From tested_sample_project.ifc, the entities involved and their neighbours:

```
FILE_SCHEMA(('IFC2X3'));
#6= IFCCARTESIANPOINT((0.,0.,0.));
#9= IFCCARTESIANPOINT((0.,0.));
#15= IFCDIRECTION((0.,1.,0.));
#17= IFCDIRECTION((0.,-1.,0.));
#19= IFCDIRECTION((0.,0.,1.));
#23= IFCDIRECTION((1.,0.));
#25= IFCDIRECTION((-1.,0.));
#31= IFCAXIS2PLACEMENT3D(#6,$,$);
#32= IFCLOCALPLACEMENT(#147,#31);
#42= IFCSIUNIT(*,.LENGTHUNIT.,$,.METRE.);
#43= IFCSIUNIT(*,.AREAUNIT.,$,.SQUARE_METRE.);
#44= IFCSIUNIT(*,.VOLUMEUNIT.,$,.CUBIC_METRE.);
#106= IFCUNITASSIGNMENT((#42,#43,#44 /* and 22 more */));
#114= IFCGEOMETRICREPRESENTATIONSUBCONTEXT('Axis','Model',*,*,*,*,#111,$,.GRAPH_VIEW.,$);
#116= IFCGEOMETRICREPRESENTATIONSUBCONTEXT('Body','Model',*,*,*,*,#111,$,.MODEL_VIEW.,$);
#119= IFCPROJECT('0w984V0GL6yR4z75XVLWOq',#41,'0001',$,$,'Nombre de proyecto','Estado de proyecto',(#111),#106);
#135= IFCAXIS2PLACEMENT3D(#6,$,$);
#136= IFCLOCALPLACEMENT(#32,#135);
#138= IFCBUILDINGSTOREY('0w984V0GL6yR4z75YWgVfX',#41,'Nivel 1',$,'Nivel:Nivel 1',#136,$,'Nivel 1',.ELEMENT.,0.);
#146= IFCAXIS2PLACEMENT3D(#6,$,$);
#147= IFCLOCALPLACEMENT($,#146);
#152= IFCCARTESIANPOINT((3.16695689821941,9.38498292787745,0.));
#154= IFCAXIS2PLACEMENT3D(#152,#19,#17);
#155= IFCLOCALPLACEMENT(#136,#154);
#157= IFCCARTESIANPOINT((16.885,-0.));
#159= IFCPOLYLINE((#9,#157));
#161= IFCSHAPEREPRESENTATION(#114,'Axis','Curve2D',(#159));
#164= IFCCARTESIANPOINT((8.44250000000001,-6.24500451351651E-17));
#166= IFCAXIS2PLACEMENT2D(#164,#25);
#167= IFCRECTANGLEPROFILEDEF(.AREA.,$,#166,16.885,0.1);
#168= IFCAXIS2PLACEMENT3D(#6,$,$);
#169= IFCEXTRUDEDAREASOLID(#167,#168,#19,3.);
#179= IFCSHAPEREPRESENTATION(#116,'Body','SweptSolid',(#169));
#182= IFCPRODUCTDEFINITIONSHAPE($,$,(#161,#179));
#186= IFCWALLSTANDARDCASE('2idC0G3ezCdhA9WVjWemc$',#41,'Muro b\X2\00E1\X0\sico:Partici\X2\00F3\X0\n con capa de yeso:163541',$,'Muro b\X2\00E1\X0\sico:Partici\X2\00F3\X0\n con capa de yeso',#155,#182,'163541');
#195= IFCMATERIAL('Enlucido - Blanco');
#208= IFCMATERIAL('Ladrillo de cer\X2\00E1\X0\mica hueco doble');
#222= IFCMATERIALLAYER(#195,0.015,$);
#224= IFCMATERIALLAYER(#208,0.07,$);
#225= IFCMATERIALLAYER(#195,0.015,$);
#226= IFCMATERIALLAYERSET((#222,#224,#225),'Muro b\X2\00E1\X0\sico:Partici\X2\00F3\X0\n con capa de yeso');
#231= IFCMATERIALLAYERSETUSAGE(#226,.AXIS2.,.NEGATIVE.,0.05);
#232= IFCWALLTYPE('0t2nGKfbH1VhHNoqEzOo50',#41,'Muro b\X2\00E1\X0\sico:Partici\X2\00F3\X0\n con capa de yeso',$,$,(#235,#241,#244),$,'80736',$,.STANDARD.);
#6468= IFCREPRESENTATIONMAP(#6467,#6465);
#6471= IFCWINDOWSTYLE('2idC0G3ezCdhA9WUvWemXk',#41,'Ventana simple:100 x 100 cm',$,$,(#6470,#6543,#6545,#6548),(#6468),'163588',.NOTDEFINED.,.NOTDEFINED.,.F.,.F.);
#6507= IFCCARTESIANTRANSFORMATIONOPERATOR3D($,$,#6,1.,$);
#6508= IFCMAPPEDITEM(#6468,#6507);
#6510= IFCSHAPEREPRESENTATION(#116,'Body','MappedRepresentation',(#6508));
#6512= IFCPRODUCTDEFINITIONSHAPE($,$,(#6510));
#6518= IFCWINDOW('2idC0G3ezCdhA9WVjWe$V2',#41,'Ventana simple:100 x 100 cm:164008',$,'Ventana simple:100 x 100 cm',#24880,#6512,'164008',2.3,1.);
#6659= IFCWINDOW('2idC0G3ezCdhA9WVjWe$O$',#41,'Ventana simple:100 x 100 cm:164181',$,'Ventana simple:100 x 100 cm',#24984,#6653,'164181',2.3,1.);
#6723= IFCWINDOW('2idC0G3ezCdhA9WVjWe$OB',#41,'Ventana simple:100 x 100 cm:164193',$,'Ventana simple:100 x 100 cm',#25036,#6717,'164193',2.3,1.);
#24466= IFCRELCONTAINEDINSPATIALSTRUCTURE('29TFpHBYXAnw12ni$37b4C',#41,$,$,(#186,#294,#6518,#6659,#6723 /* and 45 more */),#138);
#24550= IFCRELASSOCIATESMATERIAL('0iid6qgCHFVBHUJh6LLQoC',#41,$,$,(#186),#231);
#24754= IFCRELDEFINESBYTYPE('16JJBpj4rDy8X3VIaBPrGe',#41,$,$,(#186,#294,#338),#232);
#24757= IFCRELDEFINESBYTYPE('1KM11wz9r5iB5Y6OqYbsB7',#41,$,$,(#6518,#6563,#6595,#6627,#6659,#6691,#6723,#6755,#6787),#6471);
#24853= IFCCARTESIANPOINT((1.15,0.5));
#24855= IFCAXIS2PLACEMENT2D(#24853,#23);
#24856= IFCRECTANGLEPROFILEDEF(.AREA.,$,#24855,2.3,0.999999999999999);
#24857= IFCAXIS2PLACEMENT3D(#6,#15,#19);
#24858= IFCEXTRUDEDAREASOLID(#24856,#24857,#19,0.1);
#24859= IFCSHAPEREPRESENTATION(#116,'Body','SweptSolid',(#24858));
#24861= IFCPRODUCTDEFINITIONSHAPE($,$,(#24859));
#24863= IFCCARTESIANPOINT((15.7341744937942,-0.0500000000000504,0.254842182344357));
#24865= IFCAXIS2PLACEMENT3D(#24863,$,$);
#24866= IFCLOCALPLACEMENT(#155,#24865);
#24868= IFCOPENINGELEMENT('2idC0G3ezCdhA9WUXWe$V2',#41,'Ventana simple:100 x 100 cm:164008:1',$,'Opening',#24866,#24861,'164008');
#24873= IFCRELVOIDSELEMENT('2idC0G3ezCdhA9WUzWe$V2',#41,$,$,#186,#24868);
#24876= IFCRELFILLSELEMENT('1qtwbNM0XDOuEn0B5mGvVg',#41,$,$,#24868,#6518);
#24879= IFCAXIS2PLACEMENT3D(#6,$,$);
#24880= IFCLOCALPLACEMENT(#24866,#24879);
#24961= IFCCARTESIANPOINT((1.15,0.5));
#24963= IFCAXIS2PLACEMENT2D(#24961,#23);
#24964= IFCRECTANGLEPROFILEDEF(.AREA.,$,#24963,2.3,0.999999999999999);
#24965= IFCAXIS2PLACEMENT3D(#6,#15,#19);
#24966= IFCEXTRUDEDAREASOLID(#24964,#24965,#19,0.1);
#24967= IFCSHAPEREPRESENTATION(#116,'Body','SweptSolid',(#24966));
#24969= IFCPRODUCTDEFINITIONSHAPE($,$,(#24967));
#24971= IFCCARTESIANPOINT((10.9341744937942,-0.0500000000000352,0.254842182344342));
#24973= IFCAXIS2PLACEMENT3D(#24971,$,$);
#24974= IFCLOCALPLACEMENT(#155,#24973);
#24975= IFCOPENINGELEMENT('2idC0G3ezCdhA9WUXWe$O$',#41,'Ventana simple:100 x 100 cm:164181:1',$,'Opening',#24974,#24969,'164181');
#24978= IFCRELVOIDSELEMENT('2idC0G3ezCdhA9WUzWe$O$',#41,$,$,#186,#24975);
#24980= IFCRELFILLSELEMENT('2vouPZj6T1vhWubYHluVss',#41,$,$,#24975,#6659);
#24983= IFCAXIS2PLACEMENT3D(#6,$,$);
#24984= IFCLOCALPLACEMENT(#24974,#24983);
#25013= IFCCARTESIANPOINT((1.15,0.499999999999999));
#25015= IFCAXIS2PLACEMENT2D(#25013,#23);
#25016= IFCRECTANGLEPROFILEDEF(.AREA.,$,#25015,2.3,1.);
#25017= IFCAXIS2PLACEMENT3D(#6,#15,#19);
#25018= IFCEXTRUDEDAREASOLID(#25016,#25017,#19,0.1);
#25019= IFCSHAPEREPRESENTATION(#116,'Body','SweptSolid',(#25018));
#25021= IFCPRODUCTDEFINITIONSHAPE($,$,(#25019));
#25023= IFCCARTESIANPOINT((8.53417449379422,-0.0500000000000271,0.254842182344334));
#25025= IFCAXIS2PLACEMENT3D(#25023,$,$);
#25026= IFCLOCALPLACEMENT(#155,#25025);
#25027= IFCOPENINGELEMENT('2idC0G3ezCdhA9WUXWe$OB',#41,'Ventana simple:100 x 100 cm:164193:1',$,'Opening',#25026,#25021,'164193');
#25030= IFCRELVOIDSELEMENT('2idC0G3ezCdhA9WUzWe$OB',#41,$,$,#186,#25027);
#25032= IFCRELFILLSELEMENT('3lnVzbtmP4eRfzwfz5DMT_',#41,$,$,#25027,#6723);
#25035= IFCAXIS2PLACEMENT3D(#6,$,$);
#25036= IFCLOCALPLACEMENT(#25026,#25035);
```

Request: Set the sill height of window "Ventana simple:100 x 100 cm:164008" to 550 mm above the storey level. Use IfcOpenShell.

```python
import numpy as np
import ifcopenshell
import ifcopenshell.api.geometry
import ifcopenshell.geom
import ifcopenshell.util.element
import ifcopenshell.util.placement
import ifcopenshell.util.shape
import ifcopenshell.util.unit

model = ifcopenshell.open("tested_sample_project.ifc")
unit_scale = ifcopenshell.util.unit.calculate_unit_scale(model)

window = model.by_guid("2idC0G3ezCdhA9WVjWe$V2")
opening = window.FillsVoids[0].RelatingOpeningElement
storey = ifcopenshell.util.element.get_container(window, ifc_class="IfcBuildingStorey")
level = ifcopenshell.util.placement.get_local_placement(storey.ObjectPlacement)[2, 3]

# The opening's origin need not be at the sill, so measure its lowest point.
shape = ifcopenshell.geom.create_shape(ifcopenshell.geom.settings(), opening)
bottom = ifcopenshell.util.shape.get_shape_bottom_elevation(shape, shape.geometry) / unit_scale
dz = level + 0.55 / unit_scale - bottom

shift = np.array([0.0, 0.0, dz])
# The window is placed relative to its opening, so it follows when the opening moves.
matrix = ifcopenshell.util.placement.get_local_placement(opening.ObjectPlacement)
matrix[:3, 3] += shift
ifcopenshell.api.geometry.edit_object_placement(
    model, product=opening, matrix=matrix, is_si=False, should_transform_children=True
)

print(f"moved by {dz * unit_scale:+.3f} m")

model.write("tested_sample_project_rev.ifc")
```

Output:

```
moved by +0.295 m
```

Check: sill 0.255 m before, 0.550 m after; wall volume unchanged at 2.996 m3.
